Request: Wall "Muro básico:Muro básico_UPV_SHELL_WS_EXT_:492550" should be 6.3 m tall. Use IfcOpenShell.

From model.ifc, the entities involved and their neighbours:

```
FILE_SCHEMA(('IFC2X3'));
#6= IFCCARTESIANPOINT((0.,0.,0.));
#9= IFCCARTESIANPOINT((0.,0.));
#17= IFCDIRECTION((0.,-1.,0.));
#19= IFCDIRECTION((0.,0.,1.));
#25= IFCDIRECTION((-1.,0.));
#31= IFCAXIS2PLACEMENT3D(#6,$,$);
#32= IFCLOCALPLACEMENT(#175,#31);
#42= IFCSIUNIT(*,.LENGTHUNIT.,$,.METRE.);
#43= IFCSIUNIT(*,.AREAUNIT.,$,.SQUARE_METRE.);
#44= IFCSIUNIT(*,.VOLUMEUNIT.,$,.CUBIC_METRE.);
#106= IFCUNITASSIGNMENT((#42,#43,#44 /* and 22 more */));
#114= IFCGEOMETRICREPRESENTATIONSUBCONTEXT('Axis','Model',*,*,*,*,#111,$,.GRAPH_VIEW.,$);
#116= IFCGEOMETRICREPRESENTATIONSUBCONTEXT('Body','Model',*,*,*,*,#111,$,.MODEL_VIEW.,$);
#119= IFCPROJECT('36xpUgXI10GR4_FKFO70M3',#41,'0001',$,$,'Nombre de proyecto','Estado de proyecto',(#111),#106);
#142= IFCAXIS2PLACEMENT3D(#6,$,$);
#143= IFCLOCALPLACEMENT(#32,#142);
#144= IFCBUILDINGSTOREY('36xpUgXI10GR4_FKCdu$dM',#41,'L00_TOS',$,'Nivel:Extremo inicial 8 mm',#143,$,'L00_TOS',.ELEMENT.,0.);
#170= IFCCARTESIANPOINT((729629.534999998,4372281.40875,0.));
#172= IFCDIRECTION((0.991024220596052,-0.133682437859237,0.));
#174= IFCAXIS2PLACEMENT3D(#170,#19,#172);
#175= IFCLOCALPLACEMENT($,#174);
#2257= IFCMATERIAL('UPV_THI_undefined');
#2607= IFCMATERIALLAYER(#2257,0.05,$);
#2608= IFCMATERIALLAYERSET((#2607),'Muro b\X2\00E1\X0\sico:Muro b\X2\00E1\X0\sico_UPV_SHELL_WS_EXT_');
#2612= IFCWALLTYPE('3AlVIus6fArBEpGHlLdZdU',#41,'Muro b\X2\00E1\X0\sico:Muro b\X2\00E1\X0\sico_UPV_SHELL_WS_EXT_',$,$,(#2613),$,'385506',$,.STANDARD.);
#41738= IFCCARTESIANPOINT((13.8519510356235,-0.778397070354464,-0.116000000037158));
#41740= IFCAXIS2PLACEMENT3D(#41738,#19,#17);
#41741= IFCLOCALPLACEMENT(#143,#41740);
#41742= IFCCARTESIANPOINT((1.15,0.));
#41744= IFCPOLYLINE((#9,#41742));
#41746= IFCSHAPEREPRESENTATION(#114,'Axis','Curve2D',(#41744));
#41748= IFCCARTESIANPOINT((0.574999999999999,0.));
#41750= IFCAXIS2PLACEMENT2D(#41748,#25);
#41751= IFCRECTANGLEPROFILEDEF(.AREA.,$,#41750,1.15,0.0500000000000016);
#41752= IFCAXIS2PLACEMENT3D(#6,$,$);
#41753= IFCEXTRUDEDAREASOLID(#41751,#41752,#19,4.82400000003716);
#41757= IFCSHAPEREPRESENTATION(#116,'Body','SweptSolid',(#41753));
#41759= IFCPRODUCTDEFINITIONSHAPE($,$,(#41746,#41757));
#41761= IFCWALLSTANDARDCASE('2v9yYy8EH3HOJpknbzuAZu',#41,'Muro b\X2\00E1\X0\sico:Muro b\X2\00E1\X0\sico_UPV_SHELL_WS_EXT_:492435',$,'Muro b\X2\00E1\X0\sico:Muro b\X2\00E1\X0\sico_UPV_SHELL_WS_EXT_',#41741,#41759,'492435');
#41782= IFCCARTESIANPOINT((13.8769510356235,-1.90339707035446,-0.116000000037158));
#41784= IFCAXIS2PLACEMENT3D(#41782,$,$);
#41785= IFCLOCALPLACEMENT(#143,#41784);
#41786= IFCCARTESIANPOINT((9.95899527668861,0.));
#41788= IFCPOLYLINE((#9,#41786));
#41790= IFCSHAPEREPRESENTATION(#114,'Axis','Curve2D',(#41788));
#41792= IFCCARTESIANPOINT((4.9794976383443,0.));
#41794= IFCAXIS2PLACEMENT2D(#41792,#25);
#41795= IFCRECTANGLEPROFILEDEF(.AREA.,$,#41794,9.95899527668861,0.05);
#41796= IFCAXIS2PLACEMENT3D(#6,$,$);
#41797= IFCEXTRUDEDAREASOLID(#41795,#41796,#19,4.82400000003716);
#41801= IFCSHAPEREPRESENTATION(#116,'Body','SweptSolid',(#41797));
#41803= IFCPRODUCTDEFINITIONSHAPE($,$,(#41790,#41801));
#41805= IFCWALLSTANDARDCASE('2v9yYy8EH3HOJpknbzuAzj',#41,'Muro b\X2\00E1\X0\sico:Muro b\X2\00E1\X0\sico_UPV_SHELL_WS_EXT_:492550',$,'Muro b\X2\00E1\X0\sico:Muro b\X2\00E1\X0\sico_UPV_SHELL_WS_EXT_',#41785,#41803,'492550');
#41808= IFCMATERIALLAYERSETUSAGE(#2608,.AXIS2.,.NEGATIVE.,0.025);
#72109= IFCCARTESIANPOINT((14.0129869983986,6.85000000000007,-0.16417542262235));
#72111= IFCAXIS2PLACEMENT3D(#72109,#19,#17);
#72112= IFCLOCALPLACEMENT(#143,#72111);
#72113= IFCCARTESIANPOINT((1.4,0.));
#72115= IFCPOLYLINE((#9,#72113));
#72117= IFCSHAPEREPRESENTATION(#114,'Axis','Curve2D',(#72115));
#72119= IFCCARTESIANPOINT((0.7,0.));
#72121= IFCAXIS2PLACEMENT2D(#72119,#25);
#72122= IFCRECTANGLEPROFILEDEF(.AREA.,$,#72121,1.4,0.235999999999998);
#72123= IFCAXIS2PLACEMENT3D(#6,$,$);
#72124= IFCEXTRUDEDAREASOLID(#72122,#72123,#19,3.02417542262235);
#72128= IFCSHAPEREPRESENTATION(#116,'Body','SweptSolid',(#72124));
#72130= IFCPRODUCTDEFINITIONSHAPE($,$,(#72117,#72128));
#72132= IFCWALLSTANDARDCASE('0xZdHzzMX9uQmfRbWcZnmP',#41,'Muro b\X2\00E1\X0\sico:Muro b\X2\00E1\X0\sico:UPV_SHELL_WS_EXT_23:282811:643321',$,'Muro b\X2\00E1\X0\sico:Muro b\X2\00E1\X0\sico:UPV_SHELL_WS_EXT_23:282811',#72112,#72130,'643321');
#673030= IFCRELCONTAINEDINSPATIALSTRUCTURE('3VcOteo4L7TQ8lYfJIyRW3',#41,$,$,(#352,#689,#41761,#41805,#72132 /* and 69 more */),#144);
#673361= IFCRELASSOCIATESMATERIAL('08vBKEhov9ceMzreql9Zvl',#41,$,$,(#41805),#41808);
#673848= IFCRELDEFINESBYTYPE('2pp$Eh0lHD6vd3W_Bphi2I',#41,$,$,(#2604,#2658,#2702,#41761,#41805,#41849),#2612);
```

```python
import ifcopenshell
import ifcopenshell.geom
import ifcopenshell.util.representation
import ifcopenshell.util.shape

model = ifcopenshell.open("model.ifc")
settings = ifcopenshell.geom.settings()


def volume(element):
    """Net volume in cubic metres, openings subtracted."""
    shape = ifcopenshell.geom.create_shape(settings, element)
    return ifcopenshell.util.shape.get_volume(shape.geometry)


wall = model.by_id(41805)
before = volume(wall)

body = ifcopenshell.util.representation.get_representation(wall, "Model", "Body")
solid = body.Items[0]
old_height = solid.Depth
solid.Depth = 6.3
after = volume(wall)

print(f"height {old_height:g} -> {solid.Depth:g}, volume {before:.3f} -> {after:.3f} m3")

model.write("model_edited.ifc")
```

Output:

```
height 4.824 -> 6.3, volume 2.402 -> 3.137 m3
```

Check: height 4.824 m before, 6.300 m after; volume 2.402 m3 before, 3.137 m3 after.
